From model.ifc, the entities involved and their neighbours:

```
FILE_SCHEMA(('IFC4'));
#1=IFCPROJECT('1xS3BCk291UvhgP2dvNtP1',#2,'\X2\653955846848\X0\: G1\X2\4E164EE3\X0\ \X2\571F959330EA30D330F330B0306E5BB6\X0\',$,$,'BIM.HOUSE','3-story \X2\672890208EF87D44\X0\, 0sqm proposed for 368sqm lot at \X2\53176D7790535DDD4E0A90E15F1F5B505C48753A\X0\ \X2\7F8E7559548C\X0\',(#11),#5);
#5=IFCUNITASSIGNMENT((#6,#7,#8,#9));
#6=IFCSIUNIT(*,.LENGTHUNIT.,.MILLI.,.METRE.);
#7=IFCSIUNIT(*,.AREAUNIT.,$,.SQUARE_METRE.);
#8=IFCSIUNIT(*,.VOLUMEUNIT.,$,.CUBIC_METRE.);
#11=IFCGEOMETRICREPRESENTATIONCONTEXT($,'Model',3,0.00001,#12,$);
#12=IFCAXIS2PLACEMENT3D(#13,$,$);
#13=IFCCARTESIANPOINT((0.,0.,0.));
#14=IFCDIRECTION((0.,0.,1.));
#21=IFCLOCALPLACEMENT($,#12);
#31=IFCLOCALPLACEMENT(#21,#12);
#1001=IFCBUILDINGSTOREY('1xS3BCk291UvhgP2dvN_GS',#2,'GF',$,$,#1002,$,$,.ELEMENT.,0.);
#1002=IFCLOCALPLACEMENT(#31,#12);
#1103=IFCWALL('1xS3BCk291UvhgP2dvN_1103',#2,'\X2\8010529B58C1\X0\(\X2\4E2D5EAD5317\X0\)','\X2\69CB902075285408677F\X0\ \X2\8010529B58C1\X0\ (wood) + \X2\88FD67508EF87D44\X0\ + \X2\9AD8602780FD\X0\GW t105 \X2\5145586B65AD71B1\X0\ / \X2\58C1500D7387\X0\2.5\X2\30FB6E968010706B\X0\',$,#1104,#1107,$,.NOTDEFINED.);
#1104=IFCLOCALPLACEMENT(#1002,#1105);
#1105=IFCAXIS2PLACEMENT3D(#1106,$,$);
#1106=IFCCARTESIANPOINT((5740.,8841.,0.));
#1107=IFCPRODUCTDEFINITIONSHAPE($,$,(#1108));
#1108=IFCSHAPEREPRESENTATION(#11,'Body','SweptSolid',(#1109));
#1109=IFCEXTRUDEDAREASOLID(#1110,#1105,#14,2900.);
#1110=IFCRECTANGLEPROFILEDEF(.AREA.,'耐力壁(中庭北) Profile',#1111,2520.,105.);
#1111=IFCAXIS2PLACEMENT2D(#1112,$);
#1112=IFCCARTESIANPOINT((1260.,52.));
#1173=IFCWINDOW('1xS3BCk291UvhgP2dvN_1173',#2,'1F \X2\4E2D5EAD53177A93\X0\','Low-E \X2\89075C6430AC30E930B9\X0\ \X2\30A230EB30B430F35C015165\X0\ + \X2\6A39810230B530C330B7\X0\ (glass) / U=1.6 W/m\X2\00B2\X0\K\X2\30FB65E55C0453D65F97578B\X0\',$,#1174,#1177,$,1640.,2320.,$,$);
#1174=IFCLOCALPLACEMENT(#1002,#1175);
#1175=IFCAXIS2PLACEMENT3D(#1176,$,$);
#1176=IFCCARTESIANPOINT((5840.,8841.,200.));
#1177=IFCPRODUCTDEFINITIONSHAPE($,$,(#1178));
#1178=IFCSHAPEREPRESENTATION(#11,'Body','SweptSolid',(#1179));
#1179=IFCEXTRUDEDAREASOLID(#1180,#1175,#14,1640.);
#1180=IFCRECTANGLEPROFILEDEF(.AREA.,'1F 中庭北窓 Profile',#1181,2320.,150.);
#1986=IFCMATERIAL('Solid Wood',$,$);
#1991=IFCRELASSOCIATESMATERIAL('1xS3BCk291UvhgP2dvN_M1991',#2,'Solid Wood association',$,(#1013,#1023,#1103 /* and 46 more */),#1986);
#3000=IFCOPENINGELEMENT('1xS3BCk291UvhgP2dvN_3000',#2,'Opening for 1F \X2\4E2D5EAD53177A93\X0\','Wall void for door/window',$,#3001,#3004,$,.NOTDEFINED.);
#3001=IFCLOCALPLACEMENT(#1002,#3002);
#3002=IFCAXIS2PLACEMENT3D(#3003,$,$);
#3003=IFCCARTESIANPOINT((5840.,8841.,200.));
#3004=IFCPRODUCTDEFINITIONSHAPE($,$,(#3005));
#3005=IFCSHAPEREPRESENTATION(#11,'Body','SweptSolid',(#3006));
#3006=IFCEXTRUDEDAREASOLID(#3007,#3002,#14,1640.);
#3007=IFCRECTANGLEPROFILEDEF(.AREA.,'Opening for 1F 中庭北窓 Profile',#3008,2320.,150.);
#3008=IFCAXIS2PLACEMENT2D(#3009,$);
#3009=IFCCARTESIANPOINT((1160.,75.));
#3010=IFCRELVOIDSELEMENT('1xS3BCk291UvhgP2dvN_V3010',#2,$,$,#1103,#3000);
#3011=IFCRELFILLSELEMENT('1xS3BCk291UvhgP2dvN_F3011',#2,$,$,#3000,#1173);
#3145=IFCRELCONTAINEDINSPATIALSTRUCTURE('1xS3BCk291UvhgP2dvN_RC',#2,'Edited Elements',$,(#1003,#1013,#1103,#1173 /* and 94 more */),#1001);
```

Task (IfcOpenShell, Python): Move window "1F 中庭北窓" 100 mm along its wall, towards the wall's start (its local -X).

```python
import ifcopenshell
import ifcopenshell.api.geometry
import ifcopenshell.util.placement

model = ifcopenshell.open("model.ifc")

window = model.by_id(1173)
opening = window.FillsVoids[0].RelatingOpeningElement
wall = opening.VoidsElements[0].RelatingBuildingElement

wall_matrix = ifcopenshell.util.placement.get_local_placement(wall.ObjectPlacement)
shift = wall_matrix[:3, 0] * -100.0
before = ifcopenshell.util.placement.get_local_placement(window.ObjectPlacement)[:3, 3].copy()

# The window is not placed relative to its opening, so move both.
for product in (opening, window):
    matrix = ifcopenshell.util.placement.get_local_placement(product.ObjectPlacement)
    matrix[:3, 3] += shift
    ifcopenshell.api.geometry.edit_object_placement(model, product=product, matrix=matrix, is_si=False)

after = ifcopenshell.util.placement.get_local_placement(window.ObjectPlacement)[:3, 3]
print("window moved by", (after - before).round(3) + 0.0)

model.write("model_updated.ifc")
```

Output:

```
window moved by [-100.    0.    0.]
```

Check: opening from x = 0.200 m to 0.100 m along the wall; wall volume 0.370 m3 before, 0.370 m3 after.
